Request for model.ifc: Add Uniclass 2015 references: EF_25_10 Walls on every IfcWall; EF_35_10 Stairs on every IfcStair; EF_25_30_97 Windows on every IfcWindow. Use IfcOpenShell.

First a look at what the model holds.

```python
import ifcopenshell

model = ifcopenshell.open("model.ifc")
print(model.schema)
print("classifications:", [c.Name for c in model.by_type("IfcClassification")])
for ifc_class in ("IfcDoor", "IfcRoof", "IfcStair", "IfcWall", "IfcWindow"):
    print(ifc_class, len(model.by_type(ifc_class)))
```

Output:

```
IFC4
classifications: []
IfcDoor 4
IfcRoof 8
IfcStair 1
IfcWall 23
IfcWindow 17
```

```python
import ifcopenshell
import ifcopenshell.api.classification

model = ifcopenshell.open("model.ifc")

system = ifcopenshell.api.classification.add_classification(model, classification="Uniclass 2015")

codes = {
    "IfcWall": ("EF_25_10", "Walls"),
    "IfcStair": ("EF_35_10", "Stairs"),
    "IfcWindow": ("EF_25_30_97", "Windows"),
}
for ifc_class, (code, name) in codes.items():
    products = model.by_type(ifc_class)
    ifcopenshell.api.classification.add_reference(
        model, products=products, classification=system, identification=code, name=name
    )
    print(code, len(products))

model.write("model_updated.ifc")
```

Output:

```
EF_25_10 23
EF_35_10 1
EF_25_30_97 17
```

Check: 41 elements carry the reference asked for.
